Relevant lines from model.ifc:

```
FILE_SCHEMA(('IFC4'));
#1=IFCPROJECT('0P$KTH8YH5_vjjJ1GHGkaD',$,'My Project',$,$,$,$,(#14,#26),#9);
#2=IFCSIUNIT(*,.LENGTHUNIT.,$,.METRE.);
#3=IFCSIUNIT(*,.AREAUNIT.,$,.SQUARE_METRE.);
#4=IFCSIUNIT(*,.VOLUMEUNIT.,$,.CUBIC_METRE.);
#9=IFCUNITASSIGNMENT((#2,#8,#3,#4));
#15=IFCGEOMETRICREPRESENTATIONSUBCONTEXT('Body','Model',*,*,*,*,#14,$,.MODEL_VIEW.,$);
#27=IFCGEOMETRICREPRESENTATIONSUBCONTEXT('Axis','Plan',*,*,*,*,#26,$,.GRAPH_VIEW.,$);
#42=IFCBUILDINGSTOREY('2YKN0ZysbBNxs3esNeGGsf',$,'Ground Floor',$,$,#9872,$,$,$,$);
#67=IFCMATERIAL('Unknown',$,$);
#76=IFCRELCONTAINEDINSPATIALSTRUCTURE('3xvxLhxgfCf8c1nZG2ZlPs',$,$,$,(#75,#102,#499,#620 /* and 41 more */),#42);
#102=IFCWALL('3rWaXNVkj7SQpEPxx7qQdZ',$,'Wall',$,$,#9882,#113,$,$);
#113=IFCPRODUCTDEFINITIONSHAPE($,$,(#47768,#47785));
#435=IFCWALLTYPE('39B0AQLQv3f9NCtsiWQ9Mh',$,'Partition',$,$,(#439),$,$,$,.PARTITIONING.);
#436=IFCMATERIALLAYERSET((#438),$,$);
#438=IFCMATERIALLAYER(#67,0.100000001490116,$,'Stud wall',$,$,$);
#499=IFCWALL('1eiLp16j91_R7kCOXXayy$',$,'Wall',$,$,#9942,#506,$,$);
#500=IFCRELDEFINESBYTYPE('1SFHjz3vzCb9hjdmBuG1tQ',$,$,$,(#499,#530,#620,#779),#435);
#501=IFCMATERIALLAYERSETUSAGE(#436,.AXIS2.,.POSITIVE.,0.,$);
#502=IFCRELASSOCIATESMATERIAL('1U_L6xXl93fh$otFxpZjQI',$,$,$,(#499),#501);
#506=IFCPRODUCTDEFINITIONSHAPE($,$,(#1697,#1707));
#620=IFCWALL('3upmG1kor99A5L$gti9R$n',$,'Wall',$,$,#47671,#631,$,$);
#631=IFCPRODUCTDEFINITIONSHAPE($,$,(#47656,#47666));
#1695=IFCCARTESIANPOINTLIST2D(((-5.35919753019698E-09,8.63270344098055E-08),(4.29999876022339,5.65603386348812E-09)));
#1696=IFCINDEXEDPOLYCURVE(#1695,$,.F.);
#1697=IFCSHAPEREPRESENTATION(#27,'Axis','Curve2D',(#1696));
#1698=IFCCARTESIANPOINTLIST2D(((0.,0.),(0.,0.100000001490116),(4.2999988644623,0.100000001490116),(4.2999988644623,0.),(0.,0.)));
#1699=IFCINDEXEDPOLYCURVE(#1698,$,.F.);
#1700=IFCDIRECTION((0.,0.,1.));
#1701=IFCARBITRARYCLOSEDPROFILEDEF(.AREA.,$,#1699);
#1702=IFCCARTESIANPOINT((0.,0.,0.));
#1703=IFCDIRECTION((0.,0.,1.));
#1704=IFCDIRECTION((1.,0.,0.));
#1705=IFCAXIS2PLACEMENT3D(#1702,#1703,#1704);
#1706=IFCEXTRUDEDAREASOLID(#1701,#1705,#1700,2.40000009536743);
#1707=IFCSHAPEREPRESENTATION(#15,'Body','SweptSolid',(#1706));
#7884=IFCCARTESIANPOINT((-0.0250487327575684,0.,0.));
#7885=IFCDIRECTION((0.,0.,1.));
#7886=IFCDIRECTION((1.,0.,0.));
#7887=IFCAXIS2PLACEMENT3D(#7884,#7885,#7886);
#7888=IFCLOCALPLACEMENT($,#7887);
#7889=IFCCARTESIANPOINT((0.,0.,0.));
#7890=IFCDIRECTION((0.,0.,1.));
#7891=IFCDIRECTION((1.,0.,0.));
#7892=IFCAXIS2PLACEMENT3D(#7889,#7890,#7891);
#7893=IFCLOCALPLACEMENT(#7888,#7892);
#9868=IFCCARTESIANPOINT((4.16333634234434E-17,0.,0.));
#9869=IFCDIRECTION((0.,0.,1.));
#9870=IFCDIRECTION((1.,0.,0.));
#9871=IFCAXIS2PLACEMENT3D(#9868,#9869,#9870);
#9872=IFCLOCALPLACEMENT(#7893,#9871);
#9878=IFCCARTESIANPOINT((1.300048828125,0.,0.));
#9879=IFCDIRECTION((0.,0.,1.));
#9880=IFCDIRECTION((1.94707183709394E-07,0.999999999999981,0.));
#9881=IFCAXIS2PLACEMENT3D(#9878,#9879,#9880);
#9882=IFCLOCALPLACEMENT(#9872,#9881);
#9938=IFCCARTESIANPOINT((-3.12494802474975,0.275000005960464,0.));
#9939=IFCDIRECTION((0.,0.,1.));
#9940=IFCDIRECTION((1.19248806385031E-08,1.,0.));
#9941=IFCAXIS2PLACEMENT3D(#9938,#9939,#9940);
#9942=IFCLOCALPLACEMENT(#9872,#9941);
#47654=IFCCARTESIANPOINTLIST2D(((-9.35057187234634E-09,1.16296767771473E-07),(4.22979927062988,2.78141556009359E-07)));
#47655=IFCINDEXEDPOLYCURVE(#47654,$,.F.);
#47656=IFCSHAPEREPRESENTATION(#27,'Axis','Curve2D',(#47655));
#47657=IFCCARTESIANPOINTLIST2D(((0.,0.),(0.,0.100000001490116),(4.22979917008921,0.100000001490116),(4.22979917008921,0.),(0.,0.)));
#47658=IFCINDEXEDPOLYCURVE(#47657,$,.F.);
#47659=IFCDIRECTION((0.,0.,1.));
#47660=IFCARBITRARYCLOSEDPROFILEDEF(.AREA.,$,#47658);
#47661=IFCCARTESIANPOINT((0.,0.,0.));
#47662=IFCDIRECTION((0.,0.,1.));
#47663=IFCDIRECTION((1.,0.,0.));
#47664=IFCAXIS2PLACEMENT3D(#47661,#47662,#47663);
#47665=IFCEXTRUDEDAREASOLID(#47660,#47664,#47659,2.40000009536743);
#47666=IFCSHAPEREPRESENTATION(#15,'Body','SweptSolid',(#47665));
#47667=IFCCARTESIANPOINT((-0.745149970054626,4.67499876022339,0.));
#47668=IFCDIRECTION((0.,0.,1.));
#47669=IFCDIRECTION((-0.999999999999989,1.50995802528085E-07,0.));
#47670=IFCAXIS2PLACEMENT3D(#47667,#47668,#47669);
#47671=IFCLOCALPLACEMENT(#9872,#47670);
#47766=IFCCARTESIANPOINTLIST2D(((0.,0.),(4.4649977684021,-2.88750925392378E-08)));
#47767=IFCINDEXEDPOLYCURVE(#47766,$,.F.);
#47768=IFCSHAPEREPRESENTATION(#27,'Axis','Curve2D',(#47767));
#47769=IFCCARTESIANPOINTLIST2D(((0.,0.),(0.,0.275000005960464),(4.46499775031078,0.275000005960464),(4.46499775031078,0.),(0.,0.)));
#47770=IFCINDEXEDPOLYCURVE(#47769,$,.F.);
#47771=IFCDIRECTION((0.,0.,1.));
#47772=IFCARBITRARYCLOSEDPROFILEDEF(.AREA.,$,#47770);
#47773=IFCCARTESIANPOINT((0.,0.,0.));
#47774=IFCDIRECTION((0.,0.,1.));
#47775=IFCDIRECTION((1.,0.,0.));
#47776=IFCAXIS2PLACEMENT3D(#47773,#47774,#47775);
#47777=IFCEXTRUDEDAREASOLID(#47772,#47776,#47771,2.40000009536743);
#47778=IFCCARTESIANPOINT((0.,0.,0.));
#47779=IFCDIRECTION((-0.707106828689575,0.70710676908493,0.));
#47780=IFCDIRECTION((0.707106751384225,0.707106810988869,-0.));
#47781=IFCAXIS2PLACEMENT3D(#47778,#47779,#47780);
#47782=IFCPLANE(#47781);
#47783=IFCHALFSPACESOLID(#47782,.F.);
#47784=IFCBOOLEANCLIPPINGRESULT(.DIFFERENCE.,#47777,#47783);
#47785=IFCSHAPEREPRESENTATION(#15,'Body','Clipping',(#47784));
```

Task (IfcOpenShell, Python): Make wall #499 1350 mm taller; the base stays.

```python
import ifcopenshell
import ifcopenshell.geom
import ifcopenshell.util.representation
import ifcopenshell.util.shape
import ifcopenshell.util.unit

model = ifcopenshell.open("model.ifc")
unit_scale = ifcopenshell.util.unit.calculate_unit_scale(model)
settings = ifcopenshell.geom.settings()


def volume(element):
    """Net volume in cubic metres, openings subtracted."""
    shape = ifcopenshell.geom.create_shape(settings, element)
    return ifcopenshell.util.shape.get_volume(shape.geometry)


wall = model.by_guid("1eiLp16j91_R7kCOXXayy$")
before = volume(wall)

body = ifcopenshell.util.representation.get_representation(wall, "Model", "Body")
solid = body.Items[0]
old_height = solid.Depth
solid.Depth += 1.35 / unit_scale
after = volume(wall)

print(f"height {old_height:g} -> {solid.Depth:g}, volume {before:.3f} -> {after:.3f} m3")

model.write("model_updated.ifc")
```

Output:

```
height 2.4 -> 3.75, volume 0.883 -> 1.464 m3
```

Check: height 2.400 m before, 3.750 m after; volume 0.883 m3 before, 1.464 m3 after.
